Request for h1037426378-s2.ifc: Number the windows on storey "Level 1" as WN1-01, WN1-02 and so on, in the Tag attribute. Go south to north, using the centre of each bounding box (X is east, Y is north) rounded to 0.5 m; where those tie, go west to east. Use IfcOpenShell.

First a look at what the model holds.

```python
import ifcopenshell
import ifcopenshell.util.element
import ifcopenshell.util.placement

model = ifcopenshell.open("h1037426378-s2.ifc")
print(model.schema)
storey = next(s for s in model.by_type("IfcBuildingStorey") if s.Name == "Level 1")
windows = [e for e in ifcopenshell.util.element.get_decomposition(storey) if e.is_a("IfcWindow")]
for e in sorted(windows, key=lambda e: e.id()):
    origin = ifcopenshell.util.placement.get_local_placement(e.ObjectPlacement)[:3, 3]
    print(e.id(), e.Tag, e.Name, origin.round(2) + 0.0, sep=" | ")
```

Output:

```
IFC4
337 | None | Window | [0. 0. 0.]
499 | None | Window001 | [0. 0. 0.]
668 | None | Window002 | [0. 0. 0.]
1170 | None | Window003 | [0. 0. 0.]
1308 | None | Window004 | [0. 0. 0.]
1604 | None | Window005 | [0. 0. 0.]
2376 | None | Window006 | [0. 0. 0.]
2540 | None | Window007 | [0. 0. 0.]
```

```python
import ifcopenshell
import ifcopenshell.geom
import ifcopenshell.util.element
import ifcopenshell.util.shape

model = ifcopenshell.open("h1037426378-s2.ifc")
settings = ifcopenshell.geom.settings()
settings.set("use-world-coords", True)


def centre(element):
    shape = ifcopenshell.geom.create_shape(settings, element)
    return ifcopenshell.util.shape.get_bbox_centroid(shape.geometry)


storey = next(s for s in model.by_type("IfcBuildingStorey") if s.Name == "Level 1")
windows = [e for e in ifcopenshell.util.element.get_decomposition(storey) if e.is_a("IfcWindow")]

# Insertion points can sit at a corner or the storey origin, so sort by the geometry (in metres).
centres = {e: centre(e) for e in windows}
windows.sort(key=lambda e: (round(centres[e][1] / 0.5), centres[e][0]))

for i, e in enumerate(windows, start=1):
    number = f"WN1-{i:02d}"
    e.Tag = number
    print(e.id(), number)

model.write("h1037426378-s2_rev.ifc")
```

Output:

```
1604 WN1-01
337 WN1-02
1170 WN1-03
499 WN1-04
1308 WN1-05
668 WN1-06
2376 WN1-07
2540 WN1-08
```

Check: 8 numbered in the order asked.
